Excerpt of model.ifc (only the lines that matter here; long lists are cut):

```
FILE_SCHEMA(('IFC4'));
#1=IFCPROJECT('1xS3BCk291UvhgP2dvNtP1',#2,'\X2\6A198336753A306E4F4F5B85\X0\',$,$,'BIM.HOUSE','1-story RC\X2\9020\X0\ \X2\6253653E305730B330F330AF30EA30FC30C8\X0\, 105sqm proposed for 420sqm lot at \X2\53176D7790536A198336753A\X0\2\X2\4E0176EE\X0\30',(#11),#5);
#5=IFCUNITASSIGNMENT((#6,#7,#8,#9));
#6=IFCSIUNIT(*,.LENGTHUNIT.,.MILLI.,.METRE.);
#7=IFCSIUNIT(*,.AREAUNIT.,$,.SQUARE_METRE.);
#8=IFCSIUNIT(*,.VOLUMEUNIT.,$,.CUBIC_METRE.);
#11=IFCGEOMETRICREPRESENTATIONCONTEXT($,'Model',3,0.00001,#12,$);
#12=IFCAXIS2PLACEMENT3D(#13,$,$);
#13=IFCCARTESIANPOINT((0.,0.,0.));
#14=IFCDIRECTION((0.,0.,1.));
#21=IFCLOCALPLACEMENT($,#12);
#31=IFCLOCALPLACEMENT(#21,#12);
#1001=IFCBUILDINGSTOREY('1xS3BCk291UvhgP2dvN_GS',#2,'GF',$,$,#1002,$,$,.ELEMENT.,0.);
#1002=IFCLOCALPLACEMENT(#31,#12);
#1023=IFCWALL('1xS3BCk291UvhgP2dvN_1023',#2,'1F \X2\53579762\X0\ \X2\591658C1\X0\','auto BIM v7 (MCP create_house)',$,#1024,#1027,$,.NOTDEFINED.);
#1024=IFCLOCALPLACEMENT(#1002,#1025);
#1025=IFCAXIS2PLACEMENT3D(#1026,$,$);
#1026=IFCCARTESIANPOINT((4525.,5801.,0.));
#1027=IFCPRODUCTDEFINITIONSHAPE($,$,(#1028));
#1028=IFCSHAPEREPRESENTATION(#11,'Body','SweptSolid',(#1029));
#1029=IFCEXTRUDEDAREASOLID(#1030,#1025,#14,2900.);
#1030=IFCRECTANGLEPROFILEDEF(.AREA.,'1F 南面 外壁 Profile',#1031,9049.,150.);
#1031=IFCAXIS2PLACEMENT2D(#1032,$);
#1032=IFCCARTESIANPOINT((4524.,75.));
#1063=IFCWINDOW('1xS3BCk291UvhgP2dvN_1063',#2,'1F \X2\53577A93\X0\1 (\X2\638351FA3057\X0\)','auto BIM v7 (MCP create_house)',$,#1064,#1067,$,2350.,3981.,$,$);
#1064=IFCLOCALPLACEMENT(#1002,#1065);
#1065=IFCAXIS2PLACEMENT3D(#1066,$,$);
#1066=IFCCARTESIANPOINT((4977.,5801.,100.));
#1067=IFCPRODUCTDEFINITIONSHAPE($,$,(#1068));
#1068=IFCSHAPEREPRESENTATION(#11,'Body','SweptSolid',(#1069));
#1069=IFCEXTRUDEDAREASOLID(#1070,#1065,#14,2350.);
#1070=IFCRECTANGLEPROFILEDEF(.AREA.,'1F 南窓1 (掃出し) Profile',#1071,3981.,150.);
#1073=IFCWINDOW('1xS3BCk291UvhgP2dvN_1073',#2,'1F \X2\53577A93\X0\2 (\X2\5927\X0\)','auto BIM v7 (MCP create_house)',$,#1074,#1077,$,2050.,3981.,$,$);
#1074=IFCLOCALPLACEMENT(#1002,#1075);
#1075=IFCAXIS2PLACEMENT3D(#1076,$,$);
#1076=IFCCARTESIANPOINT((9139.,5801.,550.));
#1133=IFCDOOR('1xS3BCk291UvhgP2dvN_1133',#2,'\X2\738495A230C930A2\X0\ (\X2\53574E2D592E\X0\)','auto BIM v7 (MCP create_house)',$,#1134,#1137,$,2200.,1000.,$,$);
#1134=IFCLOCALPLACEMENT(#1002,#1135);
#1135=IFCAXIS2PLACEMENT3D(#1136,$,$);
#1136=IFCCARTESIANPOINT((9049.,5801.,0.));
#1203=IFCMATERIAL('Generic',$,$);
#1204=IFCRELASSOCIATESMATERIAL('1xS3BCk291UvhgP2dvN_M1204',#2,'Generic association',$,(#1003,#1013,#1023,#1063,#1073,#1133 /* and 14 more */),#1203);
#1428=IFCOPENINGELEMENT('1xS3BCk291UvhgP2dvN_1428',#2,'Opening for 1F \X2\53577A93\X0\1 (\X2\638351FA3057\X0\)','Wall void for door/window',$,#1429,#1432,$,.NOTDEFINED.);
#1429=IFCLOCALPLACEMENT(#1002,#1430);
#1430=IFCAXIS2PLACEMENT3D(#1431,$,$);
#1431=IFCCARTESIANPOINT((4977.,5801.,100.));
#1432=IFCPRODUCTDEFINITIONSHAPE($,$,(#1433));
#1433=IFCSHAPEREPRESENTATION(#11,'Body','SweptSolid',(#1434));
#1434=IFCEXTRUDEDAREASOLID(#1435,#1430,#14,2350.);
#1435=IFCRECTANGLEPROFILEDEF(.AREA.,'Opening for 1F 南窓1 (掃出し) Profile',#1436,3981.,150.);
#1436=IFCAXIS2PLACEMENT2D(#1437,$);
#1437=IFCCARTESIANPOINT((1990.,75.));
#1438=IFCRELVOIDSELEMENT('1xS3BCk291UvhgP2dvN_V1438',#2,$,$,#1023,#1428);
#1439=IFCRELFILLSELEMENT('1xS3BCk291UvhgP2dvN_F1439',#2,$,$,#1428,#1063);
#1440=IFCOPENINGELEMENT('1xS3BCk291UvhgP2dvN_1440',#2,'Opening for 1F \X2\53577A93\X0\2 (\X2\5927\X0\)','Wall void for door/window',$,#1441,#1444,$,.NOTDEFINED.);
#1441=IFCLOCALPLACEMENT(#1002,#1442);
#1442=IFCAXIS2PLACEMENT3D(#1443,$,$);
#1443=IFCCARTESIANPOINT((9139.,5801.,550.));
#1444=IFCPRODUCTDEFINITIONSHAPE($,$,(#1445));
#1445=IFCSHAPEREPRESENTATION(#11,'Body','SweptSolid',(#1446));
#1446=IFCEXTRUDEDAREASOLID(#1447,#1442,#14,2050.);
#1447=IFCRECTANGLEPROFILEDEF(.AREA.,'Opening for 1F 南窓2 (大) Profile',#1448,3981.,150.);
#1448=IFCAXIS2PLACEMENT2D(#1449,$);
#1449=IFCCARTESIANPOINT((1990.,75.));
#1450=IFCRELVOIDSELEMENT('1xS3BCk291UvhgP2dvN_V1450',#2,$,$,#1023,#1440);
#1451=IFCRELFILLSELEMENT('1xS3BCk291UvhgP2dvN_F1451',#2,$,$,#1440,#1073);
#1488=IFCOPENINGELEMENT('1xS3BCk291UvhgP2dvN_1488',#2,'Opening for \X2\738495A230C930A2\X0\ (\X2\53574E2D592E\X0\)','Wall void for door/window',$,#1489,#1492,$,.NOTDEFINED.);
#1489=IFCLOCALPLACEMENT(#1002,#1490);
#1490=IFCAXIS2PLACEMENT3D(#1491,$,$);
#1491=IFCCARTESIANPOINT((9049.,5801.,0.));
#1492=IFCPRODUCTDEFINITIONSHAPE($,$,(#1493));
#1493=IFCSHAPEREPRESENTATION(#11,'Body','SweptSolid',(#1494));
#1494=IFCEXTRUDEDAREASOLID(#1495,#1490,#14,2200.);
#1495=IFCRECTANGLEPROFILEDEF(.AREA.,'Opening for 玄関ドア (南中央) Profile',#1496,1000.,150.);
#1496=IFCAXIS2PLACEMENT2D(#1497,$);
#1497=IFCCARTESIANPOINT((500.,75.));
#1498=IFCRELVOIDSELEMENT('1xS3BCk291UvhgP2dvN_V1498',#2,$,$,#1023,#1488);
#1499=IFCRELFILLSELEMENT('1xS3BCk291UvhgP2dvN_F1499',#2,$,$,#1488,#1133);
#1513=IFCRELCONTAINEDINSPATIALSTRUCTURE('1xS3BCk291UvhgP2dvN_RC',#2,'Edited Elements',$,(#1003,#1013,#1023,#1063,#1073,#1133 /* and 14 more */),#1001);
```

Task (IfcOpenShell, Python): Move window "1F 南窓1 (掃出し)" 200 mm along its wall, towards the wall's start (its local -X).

```python
import ifcopenshell
import ifcopenshell.api.geometry
import ifcopenshell.util.placement
import ifcopenshell.util.unit

model = ifcopenshell.open("model.ifc")
unit_scale = ifcopenshell.util.unit.calculate_unit_scale(model)

window = model.by_guid("1xS3BCk291UvhgP2dvN_1063")
opening = window.FillsVoids[0].RelatingOpeningElement
wall = opening.VoidsElements[0].RelatingBuildingElement

wall_matrix = ifcopenshell.util.placement.get_local_placement(wall.ObjectPlacement)
shift = wall_matrix[:3, 0] * -0.2 / unit_scale
before = ifcopenshell.util.placement.get_local_placement(window.ObjectPlacement)[:3, 3].copy()

# The window is not placed relative to its opening, so move both.
for product in (opening, window):
    matrix = ifcopenshell.util.placement.get_local_placement(product.ObjectPlacement)
    matrix[:3, 3] += shift
    ifcopenshell.api.geometry.edit_object_placement(model, product=product, matrix=matrix, is_si=False)

after = ifcopenshell.util.placement.get_local_placement(window.ObjectPlacement)[:3, 3]
print("window moved by", (after - before).round(3) + 0.0)

model.write("model_updated.ifc")
```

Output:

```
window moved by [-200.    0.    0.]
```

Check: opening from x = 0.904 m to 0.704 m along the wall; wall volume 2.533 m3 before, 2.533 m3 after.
